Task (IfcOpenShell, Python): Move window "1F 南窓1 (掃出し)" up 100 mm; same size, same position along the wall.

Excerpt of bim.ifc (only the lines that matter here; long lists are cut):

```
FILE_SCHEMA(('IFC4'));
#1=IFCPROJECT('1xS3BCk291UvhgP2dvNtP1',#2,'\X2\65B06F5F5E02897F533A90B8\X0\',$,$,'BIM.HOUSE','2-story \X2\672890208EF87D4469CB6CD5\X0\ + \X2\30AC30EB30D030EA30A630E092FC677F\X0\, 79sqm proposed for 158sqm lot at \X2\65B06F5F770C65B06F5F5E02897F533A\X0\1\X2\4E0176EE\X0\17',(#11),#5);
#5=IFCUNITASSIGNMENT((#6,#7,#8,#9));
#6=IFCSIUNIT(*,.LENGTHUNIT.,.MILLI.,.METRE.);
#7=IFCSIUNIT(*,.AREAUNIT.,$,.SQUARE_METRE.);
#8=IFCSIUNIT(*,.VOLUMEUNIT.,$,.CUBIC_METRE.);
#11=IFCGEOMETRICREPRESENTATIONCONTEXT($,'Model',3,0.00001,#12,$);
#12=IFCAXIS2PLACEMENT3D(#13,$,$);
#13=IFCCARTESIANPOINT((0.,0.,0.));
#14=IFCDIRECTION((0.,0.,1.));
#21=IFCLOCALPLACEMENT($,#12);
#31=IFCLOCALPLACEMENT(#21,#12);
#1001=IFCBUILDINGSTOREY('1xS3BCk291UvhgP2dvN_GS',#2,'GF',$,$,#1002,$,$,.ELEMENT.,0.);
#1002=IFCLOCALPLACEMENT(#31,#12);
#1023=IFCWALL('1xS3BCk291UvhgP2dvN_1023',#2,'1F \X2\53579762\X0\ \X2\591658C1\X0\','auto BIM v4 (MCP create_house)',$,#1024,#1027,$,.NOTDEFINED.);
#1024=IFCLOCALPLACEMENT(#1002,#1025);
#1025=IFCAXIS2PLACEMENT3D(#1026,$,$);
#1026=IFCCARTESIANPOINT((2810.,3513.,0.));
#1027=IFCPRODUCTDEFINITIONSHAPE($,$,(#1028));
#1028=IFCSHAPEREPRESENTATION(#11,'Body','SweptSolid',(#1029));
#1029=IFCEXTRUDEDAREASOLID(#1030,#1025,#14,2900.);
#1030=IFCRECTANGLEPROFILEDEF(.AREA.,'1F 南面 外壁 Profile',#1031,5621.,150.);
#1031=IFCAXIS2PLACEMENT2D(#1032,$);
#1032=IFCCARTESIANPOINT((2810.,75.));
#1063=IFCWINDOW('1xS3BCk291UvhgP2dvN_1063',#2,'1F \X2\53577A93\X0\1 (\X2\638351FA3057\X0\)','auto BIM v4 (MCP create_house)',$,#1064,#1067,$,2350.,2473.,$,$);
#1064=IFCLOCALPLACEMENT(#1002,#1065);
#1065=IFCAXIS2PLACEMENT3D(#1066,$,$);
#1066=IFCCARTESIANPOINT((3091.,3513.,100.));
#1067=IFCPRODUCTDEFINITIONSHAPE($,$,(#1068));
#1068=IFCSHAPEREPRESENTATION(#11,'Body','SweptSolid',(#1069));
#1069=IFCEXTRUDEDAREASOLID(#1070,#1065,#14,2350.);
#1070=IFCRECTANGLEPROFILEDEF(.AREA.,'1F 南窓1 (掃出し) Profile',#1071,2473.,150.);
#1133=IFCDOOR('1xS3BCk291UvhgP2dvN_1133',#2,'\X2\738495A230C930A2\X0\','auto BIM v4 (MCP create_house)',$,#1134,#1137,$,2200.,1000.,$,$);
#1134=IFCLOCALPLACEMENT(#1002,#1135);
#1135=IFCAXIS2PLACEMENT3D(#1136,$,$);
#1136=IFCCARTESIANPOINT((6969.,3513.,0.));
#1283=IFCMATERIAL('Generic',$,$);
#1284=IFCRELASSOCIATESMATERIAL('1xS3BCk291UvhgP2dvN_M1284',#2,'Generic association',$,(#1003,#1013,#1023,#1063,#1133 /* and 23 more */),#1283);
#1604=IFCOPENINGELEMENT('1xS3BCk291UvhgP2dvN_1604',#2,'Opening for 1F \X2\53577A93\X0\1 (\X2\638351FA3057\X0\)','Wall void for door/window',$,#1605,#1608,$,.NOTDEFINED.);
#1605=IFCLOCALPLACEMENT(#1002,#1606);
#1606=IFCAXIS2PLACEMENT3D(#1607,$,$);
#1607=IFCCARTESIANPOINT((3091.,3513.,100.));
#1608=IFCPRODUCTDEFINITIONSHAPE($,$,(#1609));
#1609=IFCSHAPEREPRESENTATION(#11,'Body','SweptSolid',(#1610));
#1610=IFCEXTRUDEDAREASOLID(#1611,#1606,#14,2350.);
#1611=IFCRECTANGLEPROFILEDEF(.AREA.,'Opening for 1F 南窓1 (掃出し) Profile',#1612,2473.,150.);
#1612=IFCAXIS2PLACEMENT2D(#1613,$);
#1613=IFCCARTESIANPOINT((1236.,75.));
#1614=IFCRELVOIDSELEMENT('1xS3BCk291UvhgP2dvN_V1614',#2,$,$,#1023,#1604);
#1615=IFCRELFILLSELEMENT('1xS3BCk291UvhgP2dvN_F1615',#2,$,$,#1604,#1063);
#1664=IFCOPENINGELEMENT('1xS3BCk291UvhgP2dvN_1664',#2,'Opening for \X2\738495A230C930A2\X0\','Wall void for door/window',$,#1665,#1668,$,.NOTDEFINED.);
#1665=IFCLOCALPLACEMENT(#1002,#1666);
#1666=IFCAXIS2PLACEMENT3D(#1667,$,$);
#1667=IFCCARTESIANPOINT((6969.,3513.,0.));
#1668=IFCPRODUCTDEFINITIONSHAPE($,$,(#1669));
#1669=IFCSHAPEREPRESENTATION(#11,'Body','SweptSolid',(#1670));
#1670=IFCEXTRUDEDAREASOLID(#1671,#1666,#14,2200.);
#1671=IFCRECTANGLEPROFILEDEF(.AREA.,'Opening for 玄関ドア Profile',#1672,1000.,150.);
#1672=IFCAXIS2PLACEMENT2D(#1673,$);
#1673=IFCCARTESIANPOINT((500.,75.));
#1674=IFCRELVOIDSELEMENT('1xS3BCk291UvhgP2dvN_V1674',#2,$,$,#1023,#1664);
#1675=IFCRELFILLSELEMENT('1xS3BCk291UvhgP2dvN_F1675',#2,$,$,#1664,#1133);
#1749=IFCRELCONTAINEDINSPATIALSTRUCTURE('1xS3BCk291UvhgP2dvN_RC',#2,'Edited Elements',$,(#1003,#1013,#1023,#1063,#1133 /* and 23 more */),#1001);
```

```python
import numpy as np
import ifcopenshell
import ifcopenshell.api.geometry
import ifcopenshell.util.placement
import ifcopenshell.util.unit

model = ifcopenshell.open("bim.ifc")
unit_scale = ifcopenshell.util.unit.calculate_unit_scale(model)

window = model.by_guid("1xS3BCk291UvhgP2dvN_1063")
opening = window.FillsVoids[0].RelatingOpeningElement
dz = 0.1 / unit_scale

shift = np.array([0.0, 0.0, dz])
# The window is not placed relative to its opening, so move both.
for product in (opening, window):
    matrix = ifcopenshell.util.placement.get_local_placement(product.ObjectPlacement)
    matrix[:3, 3] += shift
    ifcopenshell.api.geometry.edit_object_placement(model, product=product, matrix=matrix, is_si=False)

print(f"moved by {dz * unit_scale:+.3f} m")

model.write("bim_updated.ifc")
```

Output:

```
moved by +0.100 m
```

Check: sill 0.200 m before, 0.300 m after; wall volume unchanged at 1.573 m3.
